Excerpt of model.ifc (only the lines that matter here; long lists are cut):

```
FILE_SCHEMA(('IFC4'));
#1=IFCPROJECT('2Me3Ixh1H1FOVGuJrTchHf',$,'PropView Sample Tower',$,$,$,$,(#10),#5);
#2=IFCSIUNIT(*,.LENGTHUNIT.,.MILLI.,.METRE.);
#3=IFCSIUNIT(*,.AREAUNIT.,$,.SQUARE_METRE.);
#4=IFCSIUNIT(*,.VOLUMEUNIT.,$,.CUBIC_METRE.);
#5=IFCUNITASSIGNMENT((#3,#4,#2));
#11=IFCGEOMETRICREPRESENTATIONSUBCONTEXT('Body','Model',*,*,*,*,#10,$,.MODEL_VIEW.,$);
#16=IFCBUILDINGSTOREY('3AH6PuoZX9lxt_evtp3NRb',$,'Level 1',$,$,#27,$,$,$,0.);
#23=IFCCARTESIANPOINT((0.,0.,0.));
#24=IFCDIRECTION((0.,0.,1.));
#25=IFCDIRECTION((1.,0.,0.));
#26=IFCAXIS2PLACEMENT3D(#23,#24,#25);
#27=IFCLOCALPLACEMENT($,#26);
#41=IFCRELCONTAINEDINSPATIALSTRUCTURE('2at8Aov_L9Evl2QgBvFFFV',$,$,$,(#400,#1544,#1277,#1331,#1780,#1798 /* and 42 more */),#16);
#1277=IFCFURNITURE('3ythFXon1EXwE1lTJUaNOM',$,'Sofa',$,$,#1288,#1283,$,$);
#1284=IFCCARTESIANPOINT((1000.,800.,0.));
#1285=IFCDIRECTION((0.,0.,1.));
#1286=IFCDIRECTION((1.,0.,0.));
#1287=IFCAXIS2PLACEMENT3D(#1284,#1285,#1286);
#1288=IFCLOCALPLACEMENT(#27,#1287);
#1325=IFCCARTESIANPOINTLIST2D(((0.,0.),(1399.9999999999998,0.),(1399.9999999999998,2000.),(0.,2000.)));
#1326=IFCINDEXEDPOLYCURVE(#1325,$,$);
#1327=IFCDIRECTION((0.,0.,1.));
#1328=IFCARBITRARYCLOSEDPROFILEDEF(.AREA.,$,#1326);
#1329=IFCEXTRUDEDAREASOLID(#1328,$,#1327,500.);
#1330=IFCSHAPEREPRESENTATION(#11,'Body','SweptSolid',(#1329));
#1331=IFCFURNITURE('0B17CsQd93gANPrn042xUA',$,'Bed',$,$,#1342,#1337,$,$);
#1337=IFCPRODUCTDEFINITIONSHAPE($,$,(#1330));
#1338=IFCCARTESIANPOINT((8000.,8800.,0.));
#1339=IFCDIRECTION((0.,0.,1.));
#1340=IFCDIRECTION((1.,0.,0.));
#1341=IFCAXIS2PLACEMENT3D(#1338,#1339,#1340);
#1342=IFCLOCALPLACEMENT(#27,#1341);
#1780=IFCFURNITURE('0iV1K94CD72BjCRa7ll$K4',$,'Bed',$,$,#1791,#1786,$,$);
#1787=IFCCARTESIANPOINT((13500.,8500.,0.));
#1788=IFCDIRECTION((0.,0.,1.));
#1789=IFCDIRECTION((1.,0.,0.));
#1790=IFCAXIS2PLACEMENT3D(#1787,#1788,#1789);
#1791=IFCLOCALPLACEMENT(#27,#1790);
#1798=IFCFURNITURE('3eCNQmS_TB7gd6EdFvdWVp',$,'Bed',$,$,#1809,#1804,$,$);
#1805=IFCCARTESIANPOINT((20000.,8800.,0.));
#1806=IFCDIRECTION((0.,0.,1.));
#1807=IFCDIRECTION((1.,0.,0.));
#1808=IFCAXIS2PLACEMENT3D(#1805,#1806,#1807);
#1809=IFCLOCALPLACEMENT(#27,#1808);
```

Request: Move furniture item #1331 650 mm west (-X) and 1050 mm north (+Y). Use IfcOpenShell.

```python
import ifcopenshell
import ifcopenshell.api.geometry
import ifcopenshell.util.placement

model = ifcopenshell.open("model.ifc")

item = model.by_id(1331)
matrix = ifcopenshell.util.placement.get_local_placement(item.ObjectPlacement)
matrix[0, 3] -= 650.0
matrix[1, 3] += 1050.0
ifcopenshell.api.geometry.edit_object_placement(model, product=item, matrix=matrix, is_si=False)

print(ifcopenshell.util.placement.get_local_placement(item.ObjectPlacement).round(3) + 0.0)

model.write("model_edited.ifc")
```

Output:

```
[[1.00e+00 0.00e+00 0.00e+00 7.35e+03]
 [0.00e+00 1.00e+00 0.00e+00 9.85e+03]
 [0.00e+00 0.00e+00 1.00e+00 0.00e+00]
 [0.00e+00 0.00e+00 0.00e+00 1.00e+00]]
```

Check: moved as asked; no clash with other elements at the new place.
